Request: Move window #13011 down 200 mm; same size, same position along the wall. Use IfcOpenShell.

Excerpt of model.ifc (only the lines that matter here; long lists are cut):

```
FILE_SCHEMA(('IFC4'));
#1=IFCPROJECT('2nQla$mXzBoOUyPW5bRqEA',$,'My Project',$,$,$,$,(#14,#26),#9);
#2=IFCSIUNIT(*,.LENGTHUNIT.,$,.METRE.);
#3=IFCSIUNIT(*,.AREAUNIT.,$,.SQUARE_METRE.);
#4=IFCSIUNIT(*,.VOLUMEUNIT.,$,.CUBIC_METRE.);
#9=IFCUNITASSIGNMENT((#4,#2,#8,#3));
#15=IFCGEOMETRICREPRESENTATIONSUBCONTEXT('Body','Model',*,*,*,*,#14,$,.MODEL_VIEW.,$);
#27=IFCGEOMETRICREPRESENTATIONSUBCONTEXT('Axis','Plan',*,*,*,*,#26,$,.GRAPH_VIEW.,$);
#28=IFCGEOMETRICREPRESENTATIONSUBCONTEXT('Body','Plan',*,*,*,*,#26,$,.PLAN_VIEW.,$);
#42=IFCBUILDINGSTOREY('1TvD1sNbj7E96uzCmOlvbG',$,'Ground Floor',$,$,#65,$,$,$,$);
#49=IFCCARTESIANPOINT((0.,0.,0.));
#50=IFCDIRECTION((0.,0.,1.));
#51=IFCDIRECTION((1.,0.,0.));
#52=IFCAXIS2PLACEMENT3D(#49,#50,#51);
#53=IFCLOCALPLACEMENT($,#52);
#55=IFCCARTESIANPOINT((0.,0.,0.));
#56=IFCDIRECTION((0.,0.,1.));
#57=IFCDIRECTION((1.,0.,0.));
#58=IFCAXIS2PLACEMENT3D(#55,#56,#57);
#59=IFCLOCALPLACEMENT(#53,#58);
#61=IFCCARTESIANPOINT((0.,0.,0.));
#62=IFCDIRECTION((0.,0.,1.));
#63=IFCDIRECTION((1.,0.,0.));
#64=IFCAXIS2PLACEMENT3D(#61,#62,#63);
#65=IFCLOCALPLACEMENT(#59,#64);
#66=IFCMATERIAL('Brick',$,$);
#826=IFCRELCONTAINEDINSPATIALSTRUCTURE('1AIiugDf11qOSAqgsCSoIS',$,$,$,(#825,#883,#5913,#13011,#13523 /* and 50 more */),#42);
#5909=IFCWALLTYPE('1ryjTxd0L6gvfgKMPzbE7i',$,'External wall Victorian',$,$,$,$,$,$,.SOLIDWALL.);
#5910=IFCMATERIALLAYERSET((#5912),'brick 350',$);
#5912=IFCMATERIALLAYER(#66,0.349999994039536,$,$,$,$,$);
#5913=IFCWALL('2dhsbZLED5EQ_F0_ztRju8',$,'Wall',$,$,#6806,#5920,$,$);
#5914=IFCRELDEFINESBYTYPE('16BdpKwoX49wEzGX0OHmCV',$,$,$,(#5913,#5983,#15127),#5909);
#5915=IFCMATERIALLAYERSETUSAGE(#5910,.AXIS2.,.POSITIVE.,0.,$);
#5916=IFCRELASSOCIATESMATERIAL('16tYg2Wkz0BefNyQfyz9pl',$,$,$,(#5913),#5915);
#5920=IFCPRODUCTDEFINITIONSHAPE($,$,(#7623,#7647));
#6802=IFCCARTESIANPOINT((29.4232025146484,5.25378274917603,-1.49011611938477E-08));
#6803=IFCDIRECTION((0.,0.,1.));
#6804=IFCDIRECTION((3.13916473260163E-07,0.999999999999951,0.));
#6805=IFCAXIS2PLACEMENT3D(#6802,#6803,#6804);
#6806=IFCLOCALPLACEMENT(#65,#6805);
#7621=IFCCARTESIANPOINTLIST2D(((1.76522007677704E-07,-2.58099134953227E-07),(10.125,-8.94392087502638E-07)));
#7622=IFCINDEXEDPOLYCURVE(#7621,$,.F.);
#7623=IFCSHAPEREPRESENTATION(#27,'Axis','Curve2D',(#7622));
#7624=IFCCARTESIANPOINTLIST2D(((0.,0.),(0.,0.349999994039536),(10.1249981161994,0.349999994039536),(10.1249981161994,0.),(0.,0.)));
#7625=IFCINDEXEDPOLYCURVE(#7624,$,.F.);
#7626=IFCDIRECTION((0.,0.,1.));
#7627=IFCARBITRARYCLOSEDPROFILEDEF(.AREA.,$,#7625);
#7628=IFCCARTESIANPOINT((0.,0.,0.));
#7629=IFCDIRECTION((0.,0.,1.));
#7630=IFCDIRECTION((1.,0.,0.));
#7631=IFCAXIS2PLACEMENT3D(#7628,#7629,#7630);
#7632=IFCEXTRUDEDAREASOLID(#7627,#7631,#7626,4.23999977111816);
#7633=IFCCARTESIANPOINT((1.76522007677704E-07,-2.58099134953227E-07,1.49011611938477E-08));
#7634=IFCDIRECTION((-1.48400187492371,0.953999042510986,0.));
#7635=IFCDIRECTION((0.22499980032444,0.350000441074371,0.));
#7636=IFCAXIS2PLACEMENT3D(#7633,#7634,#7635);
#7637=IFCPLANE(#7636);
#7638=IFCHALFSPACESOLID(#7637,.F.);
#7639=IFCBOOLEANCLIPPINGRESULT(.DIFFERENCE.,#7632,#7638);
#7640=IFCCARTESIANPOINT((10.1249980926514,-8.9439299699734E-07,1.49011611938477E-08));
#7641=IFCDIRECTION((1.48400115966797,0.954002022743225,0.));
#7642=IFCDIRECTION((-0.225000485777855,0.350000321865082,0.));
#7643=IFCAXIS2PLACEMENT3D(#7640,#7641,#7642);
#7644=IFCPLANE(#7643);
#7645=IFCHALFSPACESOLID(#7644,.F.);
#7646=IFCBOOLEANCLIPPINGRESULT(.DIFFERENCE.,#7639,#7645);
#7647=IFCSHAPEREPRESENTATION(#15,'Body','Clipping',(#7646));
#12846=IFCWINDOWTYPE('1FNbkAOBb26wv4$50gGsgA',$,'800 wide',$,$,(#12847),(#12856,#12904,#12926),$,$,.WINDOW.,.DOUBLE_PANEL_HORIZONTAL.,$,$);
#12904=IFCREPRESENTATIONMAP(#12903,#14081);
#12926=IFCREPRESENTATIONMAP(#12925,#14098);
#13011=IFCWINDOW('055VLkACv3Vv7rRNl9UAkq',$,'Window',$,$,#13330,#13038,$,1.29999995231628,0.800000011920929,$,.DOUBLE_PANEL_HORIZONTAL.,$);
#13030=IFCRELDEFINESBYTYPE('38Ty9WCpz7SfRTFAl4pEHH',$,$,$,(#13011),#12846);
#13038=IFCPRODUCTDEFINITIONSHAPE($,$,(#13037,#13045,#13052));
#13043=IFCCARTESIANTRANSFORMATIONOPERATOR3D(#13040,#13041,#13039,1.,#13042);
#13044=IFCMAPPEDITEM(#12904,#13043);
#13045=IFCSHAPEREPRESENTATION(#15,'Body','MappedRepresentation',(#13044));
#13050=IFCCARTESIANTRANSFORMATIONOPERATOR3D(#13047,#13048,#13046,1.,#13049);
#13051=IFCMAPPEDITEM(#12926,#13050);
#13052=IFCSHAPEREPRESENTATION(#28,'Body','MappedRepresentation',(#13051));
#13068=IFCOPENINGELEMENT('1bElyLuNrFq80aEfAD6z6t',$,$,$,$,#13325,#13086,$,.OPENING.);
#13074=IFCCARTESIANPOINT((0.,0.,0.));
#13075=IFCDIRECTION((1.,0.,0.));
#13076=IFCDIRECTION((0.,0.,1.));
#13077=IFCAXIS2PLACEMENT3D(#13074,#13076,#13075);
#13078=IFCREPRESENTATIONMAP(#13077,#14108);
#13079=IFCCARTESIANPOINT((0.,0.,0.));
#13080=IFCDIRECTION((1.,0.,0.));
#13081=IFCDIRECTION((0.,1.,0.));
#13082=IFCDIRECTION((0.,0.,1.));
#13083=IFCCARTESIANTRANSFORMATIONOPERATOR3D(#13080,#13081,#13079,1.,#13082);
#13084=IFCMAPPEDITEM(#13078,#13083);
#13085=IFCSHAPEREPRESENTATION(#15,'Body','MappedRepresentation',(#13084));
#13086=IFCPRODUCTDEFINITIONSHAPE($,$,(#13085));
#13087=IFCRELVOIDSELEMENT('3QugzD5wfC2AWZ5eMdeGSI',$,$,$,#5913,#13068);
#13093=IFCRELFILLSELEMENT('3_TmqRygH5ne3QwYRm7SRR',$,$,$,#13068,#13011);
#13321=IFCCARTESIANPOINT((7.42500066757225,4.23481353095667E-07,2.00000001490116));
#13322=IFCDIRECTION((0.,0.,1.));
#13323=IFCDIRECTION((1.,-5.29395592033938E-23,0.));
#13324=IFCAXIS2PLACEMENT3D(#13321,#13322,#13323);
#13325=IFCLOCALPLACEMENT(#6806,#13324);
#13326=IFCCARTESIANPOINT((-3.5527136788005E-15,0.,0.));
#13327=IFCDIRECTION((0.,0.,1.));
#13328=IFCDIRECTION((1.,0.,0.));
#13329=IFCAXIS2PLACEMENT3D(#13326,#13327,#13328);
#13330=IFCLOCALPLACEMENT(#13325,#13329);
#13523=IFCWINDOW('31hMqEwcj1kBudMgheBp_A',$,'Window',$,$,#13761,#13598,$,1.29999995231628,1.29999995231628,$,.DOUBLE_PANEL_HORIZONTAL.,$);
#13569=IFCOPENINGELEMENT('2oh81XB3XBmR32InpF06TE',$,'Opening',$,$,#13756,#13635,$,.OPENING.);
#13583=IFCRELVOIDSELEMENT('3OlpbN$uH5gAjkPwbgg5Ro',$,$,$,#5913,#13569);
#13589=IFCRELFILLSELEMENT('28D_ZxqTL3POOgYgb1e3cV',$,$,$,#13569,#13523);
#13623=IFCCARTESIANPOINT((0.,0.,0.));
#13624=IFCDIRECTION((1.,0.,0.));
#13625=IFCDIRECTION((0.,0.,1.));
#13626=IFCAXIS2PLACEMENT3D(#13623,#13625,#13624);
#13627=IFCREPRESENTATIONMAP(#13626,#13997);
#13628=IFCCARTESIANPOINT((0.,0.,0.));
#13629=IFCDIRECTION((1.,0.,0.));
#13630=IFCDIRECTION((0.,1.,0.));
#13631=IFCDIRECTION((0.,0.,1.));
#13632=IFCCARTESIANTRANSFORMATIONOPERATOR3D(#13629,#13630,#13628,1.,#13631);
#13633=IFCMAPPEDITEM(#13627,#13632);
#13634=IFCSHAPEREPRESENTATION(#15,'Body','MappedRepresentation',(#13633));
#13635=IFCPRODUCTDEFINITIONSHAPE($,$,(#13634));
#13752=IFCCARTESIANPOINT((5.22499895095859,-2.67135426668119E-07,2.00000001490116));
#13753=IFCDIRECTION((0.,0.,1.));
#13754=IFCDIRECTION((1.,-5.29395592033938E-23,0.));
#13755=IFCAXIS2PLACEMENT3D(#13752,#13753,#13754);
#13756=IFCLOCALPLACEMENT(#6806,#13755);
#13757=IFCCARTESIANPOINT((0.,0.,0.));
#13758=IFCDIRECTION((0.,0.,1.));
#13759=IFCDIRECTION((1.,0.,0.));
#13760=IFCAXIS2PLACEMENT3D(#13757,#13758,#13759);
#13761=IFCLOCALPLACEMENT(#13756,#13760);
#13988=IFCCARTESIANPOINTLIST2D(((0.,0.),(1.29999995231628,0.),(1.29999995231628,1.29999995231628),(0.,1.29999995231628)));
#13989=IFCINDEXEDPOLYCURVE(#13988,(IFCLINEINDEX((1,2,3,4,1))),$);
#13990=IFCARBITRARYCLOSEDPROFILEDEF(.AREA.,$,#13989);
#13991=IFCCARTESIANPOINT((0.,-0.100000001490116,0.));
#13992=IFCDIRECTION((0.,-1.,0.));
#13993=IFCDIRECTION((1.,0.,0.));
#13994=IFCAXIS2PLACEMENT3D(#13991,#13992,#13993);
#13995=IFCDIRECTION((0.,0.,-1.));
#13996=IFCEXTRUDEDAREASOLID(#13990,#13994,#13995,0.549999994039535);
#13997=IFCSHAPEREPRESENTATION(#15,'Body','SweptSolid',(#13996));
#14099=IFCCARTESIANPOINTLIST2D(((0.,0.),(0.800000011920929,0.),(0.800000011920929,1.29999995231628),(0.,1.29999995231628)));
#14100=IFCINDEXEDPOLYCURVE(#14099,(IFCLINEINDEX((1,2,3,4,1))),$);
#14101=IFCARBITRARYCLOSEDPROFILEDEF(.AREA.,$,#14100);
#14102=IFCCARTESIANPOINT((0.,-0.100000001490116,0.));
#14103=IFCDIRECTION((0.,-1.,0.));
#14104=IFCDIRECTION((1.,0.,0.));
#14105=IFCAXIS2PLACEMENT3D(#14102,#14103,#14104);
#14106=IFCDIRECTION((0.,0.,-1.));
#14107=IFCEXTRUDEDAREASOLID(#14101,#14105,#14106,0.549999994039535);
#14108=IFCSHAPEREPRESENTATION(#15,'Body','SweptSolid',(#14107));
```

```python
import numpy as np
import ifcopenshell
import ifcopenshell.api.geometry
import ifcopenshell.util.placement
import ifcopenshell.util.unit

model = ifcopenshell.open("model.ifc")
unit_scale = ifcopenshell.util.unit.calculate_unit_scale(model)

window = model.by_guid("055VLkACv3Vv7rRNl9UAkq")
opening = window.FillsVoids[0].RelatingOpeningElement
dz = -0.2

shift = np.array([0.0, 0.0, dz])
# The window is placed relative to its opening, so it follows when the opening moves.
matrix = ifcopenshell.util.placement.get_local_placement(opening.ObjectPlacement)
matrix[:3, 3] += shift
ifcopenshell.api.geometry.edit_object_placement(
    model, product=opening, matrix=matrix, is_si=False, should_transform_children=True
)

print(f"moved by {dz * unit_scale:+.3f} m")

model.write("model_rev.ifc")
```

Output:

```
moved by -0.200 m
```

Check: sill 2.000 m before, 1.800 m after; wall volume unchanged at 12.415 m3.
